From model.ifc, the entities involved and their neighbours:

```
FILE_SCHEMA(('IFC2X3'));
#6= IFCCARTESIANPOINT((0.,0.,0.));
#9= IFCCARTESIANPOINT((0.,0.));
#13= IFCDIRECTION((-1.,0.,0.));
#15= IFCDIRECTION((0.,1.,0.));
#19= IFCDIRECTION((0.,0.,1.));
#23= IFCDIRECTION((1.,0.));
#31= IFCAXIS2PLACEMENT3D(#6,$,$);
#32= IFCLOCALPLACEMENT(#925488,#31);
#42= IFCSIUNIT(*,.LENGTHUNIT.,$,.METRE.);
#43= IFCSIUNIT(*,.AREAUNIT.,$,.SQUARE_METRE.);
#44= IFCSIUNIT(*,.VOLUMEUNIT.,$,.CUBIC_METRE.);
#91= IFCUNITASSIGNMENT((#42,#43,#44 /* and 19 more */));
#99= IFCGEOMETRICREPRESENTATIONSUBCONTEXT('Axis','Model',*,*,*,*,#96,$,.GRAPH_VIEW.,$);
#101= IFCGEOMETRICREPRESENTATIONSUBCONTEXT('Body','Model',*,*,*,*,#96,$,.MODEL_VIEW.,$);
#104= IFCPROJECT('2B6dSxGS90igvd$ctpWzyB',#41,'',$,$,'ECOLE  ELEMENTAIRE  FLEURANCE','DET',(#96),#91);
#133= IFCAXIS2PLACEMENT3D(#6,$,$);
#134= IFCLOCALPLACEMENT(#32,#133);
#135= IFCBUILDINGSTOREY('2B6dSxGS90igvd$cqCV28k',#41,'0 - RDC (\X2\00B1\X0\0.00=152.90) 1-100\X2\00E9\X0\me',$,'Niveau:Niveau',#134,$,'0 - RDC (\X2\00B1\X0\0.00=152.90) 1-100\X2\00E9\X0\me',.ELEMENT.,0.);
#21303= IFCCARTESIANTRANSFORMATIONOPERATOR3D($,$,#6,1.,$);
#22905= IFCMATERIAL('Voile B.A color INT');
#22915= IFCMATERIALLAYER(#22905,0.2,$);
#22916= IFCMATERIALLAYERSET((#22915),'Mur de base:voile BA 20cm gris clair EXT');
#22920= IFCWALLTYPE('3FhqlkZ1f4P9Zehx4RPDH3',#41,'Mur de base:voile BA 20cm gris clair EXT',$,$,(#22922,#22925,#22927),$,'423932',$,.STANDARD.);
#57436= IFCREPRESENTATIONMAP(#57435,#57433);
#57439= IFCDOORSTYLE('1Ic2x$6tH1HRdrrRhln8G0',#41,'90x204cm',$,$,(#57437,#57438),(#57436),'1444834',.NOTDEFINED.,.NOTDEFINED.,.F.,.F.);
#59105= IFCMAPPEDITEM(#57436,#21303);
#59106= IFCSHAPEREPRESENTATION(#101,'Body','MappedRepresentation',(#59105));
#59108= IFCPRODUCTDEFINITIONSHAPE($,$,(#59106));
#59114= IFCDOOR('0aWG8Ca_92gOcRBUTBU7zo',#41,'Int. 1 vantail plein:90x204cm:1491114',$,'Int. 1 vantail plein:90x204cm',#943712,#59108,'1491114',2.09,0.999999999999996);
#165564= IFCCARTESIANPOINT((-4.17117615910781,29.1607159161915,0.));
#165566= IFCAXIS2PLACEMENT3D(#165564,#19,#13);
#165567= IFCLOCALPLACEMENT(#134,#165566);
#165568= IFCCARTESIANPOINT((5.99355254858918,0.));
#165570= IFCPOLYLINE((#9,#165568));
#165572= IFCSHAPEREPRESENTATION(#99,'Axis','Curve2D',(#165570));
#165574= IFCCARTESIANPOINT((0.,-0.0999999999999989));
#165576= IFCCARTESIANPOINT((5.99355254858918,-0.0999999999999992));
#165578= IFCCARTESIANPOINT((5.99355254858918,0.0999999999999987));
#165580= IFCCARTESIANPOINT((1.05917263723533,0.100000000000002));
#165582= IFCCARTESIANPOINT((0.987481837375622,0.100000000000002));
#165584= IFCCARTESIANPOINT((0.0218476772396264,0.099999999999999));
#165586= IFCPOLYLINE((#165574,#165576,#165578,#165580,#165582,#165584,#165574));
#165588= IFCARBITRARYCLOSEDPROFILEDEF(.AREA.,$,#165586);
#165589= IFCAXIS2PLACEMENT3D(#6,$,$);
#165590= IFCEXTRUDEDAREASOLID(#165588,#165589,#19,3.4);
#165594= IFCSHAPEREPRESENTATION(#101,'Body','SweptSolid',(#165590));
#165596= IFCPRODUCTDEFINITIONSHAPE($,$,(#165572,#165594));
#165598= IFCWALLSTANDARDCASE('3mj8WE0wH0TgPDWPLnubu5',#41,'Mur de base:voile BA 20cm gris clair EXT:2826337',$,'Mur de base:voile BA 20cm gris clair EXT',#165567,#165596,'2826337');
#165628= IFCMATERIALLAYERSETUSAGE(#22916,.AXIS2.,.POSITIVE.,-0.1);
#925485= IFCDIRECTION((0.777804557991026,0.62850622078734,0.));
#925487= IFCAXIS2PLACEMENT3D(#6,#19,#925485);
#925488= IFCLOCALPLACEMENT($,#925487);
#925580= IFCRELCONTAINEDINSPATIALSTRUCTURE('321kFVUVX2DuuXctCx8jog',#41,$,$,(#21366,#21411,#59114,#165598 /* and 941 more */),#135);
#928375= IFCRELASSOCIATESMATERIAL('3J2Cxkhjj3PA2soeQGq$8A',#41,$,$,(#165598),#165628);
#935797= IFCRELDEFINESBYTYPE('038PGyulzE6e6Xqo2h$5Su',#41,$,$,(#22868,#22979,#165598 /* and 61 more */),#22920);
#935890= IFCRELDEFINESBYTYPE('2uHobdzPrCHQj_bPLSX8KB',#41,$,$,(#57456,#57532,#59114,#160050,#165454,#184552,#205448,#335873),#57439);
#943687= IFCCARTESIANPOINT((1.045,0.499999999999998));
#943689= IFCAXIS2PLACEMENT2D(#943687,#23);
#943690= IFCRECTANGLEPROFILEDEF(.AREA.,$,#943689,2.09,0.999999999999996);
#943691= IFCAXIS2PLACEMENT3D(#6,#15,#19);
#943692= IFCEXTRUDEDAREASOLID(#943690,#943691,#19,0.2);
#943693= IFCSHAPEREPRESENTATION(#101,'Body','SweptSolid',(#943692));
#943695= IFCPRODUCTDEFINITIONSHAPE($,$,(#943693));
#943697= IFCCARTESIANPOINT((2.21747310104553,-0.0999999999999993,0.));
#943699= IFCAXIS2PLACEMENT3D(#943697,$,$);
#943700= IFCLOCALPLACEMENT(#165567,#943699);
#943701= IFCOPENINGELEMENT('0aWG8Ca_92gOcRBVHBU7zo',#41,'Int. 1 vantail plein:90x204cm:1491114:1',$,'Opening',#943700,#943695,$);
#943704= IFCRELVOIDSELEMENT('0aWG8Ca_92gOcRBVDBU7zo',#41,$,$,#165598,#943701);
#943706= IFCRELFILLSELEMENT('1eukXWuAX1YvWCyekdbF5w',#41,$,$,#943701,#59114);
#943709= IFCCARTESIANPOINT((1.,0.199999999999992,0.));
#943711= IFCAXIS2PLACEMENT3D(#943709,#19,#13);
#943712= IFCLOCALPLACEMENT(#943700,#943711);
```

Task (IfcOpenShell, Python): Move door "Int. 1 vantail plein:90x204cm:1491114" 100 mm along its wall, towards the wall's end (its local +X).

```python
import ifcopenshell
import ifcopenshell.api.geometry
import ifcopenshell.util.placement

model = ifcopenshell.open("model.ifc")

door = model.by_guid("0aWG8Ca_92gOcRBUTBU7zo")
opening = door.FillsVoids[0].RelatingOpeningElement
wall = opening.VoidsElements[0].RelatingBuildingElement

wall_matrix = ifcopenshell.util.placement.get_local_placement(wall.ObjectPlacement)
shift = wall_matrix[:3, 0] * 0.1
before = ifcopenshell.util.placement.get_local_placement(door.ObjectPlacement)[:3, 3].copy()

# The door is placed relative to its opening, so it follows when the opening moves.
matrix = ifcopenshell.util.placement.get_local_placement(opening.ObjectPlacement)
matrix[:3, 3] += shift
ifcopenshell.api.geometry.edit_object_placement(
    model, product=opening, matrix=matrix, is_si=False, should_transform_children=True
)

after = ifcopenshell.util.placement.get_local_placement(door.ObjectPlacement)[:3, 3]
print("door moved by", (after - before).round(3) + 0.0)

model.write("model_updated.ifc")
```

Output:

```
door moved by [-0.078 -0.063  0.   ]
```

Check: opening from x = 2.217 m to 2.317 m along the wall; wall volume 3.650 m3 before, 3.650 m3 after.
